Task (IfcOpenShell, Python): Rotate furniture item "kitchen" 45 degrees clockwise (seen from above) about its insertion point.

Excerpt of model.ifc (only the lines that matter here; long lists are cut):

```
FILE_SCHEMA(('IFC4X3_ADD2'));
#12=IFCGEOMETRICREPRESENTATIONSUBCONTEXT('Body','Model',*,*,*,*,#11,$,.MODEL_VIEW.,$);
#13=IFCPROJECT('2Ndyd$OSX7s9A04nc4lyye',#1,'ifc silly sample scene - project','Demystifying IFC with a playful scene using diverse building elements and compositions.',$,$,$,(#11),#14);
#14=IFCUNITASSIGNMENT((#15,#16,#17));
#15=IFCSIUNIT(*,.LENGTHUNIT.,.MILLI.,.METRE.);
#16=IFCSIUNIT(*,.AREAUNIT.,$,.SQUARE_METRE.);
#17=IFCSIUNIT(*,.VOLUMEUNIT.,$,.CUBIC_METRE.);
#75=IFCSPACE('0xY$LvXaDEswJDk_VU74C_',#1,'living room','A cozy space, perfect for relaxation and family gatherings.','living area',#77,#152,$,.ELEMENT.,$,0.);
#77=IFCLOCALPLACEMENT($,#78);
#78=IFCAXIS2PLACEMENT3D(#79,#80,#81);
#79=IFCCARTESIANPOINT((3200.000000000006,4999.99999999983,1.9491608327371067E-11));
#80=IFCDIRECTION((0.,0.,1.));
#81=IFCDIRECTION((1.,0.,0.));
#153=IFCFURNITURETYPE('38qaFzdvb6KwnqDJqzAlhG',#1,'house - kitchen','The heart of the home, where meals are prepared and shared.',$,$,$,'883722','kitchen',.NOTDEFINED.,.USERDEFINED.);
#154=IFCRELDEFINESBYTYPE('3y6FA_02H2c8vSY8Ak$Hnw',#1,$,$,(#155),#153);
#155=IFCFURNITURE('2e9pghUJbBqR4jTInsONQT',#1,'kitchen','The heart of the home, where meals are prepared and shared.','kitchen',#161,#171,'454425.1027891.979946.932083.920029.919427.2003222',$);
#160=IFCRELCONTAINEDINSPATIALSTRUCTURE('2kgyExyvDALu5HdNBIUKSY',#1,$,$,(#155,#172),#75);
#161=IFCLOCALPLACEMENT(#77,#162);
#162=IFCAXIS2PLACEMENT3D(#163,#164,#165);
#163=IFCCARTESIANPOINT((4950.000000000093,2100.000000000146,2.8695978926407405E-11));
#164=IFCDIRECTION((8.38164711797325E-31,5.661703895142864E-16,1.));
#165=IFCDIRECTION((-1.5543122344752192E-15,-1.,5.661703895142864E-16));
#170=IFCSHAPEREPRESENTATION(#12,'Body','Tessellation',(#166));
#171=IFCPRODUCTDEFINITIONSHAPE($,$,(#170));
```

```python
import ifcopenshell
import ifcopenshell.api.geometry
import ifcopenshell.util.placement

model = ifcopenshell.open("model.ifc")

item = model.by_guid("2e9pghUJbBqR4jTInsONQT")
matrix = ifcopenshell.util.placement.get_local_placement(item.ObjectPlacement)
matrix = matrix @ ifcopenshell.util.placement.rotation(-45, "Z")
ifcopenshell.api.geometry.edit_object_placement(model, product=item, matrix=matrix, is_si=False)

print(ifcopenshell.util.placement.get_local_placement(item.ObjectPlacement).round(3) + 0.0)

model.write("model_v2.ifc")
```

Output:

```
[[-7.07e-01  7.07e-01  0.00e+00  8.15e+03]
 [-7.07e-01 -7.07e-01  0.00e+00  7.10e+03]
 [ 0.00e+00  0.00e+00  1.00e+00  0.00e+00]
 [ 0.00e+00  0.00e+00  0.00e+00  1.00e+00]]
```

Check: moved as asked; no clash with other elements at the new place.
